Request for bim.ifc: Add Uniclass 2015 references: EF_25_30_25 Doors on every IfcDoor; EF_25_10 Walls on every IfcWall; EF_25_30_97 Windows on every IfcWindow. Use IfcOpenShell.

First a look at what the model holds.

```python
import ifcopenshell

model = ifcopenshell.open("bim.ifc")
print(model.schema)
print("classifications:", [c.Name for c in model.by_type("IfcClassification")])
for ifc_class in ("IfcDoor", "IfcRoof", "IfcStair", "IfcWall", "IfcWindow"):
    print(ifc_class, len(model.by_type(ifc_class)))
```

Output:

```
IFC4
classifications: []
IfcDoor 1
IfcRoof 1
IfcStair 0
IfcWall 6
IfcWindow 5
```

```python
import ifcopenshell
import ifcopenshell.api.classification

model = ifcopenshell.open("bim.ifc")

system = ifcopenshell.api.classification.add_classification(model, classification="Uniclass 2015")

codes = {
    "IfcDoor": ("EF_25_30_25", "Doors"),
    "IfcWall": ("EF_25_10", "Walls"),
    "IfcWindow": ("EF_25_30_97", "Windows"),
}
for ifc_class, (code, name) in codes.items():
    products = model.by_type(ifc_class)
    ifcopenshell.api.classification.add_reference(
        model, products=products, classification=system, identification=code, name=name
    )
    print(code, len(products))

model.write("bim-out.ifc")
```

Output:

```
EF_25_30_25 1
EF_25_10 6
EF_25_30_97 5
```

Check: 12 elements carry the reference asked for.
